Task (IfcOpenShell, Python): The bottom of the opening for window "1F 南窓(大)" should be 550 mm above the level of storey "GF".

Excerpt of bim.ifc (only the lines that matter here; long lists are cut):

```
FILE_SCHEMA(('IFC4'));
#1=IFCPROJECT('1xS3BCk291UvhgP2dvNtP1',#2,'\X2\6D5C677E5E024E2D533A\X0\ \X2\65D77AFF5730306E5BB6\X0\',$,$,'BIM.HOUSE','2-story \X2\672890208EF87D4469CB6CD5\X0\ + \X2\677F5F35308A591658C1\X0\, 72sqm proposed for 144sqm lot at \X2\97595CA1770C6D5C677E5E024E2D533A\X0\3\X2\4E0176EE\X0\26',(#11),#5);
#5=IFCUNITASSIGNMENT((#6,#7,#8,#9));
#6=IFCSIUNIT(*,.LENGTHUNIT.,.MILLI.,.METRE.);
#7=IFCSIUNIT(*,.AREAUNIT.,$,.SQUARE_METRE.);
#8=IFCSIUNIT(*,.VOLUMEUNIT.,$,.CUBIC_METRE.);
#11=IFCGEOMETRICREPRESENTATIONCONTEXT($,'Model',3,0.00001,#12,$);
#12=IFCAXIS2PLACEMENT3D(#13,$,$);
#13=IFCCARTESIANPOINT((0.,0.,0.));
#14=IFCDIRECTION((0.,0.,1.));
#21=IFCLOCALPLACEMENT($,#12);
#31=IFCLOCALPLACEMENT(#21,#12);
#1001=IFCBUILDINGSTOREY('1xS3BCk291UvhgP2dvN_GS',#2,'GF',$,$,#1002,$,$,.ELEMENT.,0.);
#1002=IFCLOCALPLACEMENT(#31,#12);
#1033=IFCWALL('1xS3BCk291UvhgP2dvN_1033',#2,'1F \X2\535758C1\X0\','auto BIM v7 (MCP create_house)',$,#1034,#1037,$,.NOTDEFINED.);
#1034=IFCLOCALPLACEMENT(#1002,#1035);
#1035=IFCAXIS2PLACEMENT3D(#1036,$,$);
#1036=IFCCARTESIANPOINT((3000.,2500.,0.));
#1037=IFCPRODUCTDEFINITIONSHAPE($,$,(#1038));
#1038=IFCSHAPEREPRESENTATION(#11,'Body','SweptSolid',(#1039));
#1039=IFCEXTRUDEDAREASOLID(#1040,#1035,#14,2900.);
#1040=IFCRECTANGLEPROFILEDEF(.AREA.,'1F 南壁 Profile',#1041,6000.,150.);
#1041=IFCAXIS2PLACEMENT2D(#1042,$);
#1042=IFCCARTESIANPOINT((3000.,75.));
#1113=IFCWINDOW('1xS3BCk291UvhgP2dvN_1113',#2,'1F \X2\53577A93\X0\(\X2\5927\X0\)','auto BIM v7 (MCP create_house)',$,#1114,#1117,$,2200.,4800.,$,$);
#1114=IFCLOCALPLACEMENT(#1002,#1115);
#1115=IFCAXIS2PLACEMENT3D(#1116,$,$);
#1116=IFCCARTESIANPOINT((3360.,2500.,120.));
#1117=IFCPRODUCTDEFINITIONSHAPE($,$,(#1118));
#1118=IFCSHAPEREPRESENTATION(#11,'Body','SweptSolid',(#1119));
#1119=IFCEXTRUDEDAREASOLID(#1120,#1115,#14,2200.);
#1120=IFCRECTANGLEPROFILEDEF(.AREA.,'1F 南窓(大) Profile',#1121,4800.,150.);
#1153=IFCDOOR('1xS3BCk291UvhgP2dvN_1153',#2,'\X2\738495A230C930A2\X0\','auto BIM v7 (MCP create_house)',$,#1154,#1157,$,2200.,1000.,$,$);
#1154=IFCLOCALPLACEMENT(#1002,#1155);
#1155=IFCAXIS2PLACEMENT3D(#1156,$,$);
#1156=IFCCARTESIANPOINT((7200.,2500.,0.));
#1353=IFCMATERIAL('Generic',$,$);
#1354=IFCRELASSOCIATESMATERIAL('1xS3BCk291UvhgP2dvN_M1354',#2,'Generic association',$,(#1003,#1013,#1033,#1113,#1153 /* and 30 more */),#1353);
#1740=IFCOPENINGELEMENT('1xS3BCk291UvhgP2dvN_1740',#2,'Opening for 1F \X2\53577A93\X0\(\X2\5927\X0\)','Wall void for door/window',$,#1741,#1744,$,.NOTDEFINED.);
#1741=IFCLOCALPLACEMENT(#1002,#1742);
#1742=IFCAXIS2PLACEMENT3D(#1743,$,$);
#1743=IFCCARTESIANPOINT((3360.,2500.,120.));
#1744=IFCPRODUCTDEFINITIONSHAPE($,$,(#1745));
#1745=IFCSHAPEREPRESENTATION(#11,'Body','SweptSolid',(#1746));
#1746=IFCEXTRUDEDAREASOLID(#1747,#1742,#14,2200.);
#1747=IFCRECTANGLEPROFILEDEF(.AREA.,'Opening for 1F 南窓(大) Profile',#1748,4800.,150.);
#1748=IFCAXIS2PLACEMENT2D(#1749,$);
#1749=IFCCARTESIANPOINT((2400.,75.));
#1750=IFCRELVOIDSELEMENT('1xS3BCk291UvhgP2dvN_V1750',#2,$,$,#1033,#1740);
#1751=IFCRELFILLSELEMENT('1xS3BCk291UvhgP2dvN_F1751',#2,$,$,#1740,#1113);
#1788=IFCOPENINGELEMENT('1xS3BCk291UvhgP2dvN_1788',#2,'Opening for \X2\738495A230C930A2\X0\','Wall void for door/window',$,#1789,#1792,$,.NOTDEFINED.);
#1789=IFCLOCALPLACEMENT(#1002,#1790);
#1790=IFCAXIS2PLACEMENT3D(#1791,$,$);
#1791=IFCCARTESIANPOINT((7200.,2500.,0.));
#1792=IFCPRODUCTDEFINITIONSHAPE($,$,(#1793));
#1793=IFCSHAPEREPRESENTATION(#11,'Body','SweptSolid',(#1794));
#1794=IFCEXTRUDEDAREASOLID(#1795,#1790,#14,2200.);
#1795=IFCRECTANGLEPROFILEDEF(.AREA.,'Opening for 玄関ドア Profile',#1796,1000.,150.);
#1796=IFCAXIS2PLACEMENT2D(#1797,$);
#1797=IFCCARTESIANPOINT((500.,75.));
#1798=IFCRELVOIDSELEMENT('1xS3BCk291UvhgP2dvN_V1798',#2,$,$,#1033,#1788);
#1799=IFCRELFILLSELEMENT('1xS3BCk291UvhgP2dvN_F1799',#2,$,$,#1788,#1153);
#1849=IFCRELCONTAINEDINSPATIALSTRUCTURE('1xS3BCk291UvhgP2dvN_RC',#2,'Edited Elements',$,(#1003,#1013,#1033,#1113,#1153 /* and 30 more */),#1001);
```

```python
import numpy as np
import ifcopenshell
import ifcopenshell.api.geometry
import ifcopenshell.geom
import ifcopenshell.util.element
import ifcopenshell.util.placement
import ifcopenshell.util.shape
import ifcopenshell.util.unit

model = ifcopenshell.open("bim.ifc")
unit_scale = ifcopenshell.util.unit.calculate_unit_scale(model)

window = model.by_guid("1xS3BCk291UvhgP2dvN_1113")
opening = window.FillsVoids[0].RelatingOpeningElement
storey = ifcopenshell.util.element.get_container(window, ifc_class="IfcBuildingStorey")
level = ifcopenshell.util.placement.get_local_placement(storey.ObjectPlacement)[2, 3]

# The opening's origin need not be at the sill, so measure its lowest point.
shape = ifcopenshell.geom.create_shape(ifcopenshell.geom.settings(), opening)
bottom = ifcopenshell.util.shape.get_shape_bottom_elevation(shape, shape.geometry) / unit_scale
dz = level + 0.55 / unit_scale - bottom

shift = np.array([0.0, 0.0, dz])
# The window is not placed relative to its opening, so move both.
for product in (opening, window):
    matrix = ifcopenshell.util.placement.get_local_placement(product.ObjectPlacement)
    matrix[:3, 3] += shift
    ifcopenshell.api.geometry.edit_object_placement(model, product=product, matrix=matrix, is_si=False)

print(f"moved by {dz * unit_scale:+.3f} m")

model.write("bim_updated.ifc")
```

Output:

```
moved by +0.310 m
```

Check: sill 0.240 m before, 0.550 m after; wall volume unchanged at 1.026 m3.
